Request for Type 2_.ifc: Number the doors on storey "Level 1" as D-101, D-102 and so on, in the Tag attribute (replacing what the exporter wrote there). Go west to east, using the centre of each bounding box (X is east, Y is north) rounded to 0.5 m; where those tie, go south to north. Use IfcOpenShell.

First a look at what the model holds.

```python
import ifcopenshell
import ifcopenshell.util.element
import ifcopenshell.util.placement

model = ifcopenshell.open("Type 2_.ifc")
print(model.schema)
storey = next(s for s in model.by_type("IfcBuildingStorey") if s.Name == "Level 1")
doors = [e for e in ifcopenshell.util.element.get_decomposition(storey) if e.is_a("IfcDoor")]
for e in sorted(doors, key=lambda e: e.id()):
    origin = ifcopenshell.util.placement.get_local_placement(e.ObjectPlacement)[:3, 3]
    print(e.id(), e.Tag, e.Name, origin.round(2) + 0.0, sep=" | ")
```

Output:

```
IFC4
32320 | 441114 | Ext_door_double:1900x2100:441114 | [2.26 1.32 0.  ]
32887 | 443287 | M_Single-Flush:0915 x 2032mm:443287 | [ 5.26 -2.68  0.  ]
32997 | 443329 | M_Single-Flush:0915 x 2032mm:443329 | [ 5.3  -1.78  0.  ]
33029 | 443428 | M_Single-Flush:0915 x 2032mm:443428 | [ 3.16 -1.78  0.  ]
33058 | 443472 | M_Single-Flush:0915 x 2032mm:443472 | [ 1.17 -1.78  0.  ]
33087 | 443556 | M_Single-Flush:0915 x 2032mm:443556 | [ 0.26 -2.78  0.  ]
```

```python
import ifcopenshell
import ifcopenshell.geom
import ifcopenshell.util.element
import ifcopenshell.util.shape

model = ifcopenshell.open("Type 2_.ifc")
settings = ifcopenshell.geom.settings()
settings.set("use-world-coords", True)


def centre(element):
    shape = ifcopenshell.geom.create_shape(settings, element)
    return ifcopenshell.util.shape.get_bbox_centroid(shape.geometry)


storey = next(s for s in model.by_type("IfcBuildingStorey") if s.Name == "Level 1")
doors = [e for e in ifcopenshell.util.element.get_decomposition(storey) if e.is_a("IfcDoor")]

# Insertion points can sit at a corner or the storey origin, so sort by the geometry (in metres).
centres = {e: centre(e) for e in doors}
doors.sort(key=lambda e: (round(centres[e][0] / 0.5), centres[e][1]))

for i, e in enumerate(doors, start=1):
    number = f"D-1{i:02d}"
    e.Tag = number
    print(e.id(), number)

model.write("Type 2__rev.ifc")
```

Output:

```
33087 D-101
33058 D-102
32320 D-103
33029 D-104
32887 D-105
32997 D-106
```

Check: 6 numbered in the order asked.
